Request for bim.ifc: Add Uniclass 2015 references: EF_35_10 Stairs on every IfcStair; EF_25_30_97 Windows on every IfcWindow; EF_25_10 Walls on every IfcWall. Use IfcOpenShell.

First a look at what the model holds.

```python
import ifcopenshell

model = ifcopenshell.open("bim.ifc")
print(model.schema)
print("classifications:", [c.Name for c in model.by_type("IfcClassification")])
for ifc_class in ("IfcDoor", "IfcRoof", "IfcStair", "IfcWall", "IfcWindow"):
    print(ifc_class, len(model.by_type(ifc_class)))
```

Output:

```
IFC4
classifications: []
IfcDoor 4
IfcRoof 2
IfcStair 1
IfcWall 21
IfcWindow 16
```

```python
import ifcopenshell
import ifcopenshell.api.classification

model = ifcopenshell.open("bim.ifc")

system = ifcopenshell.api.classification.add_classification(model, classification="Uniclass 2015")

codes = {
    "IfcStair": ("EF_35_10", "Stairs"),
    "IfcWindow": ("EF_25_30_97", "Windows"),
    "IfcWall": ("EF_25_10", "Walls"),
}
for ifc_class, (code, name) in codes.items():
    products = model.by_type(ifc_class)
    ifcopenshell.api.classification.add_reference(
        model, products=products, classification=system, identification=code, name=name
    )
    print(code, len(products))

model.write("bim_updated.ifc")
```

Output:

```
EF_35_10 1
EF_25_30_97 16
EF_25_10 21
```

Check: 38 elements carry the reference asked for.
